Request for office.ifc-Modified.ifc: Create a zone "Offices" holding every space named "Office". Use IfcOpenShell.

First a look at what the model holds.

```python
import ifcopenshell

model = ifcopenshell.open("office.ifc-Modified.ifc")
print(model.schema)
seen = {}
for space in model.by_type("IfcSpace"):
    seen[space.LongName] = seen.get(space.LongName, 0) + 1
for name, count in sorted(seen.items(), key=str):
    print(count, "x", name)
print("zones:", [z.Name for z in model.by_type("IfcZone")][:20])
```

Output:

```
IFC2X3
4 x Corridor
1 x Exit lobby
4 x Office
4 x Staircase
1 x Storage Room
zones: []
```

```python
import ifcopenshell
import ifcopenshell.api.group
import ifcopenshell.api.root

model = ifcopenshell.open("office.ifc-Modified.ifc")

names = {"Office"}
spaces = [s for s in model.by_type("IfcSpace") if s.LongName in names]

zone = ifcopenshell.api.root.create_entity(model, ifc_class="IfcZone", name="Offices")
ifcopenshell.api.group.assign_group(model, products=spaces, group=zone)
print(len(spaces), "spaces in", zone.Name)

model.write("office.ifc-Modified-out.ifc")
```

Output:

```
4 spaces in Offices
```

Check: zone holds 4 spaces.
